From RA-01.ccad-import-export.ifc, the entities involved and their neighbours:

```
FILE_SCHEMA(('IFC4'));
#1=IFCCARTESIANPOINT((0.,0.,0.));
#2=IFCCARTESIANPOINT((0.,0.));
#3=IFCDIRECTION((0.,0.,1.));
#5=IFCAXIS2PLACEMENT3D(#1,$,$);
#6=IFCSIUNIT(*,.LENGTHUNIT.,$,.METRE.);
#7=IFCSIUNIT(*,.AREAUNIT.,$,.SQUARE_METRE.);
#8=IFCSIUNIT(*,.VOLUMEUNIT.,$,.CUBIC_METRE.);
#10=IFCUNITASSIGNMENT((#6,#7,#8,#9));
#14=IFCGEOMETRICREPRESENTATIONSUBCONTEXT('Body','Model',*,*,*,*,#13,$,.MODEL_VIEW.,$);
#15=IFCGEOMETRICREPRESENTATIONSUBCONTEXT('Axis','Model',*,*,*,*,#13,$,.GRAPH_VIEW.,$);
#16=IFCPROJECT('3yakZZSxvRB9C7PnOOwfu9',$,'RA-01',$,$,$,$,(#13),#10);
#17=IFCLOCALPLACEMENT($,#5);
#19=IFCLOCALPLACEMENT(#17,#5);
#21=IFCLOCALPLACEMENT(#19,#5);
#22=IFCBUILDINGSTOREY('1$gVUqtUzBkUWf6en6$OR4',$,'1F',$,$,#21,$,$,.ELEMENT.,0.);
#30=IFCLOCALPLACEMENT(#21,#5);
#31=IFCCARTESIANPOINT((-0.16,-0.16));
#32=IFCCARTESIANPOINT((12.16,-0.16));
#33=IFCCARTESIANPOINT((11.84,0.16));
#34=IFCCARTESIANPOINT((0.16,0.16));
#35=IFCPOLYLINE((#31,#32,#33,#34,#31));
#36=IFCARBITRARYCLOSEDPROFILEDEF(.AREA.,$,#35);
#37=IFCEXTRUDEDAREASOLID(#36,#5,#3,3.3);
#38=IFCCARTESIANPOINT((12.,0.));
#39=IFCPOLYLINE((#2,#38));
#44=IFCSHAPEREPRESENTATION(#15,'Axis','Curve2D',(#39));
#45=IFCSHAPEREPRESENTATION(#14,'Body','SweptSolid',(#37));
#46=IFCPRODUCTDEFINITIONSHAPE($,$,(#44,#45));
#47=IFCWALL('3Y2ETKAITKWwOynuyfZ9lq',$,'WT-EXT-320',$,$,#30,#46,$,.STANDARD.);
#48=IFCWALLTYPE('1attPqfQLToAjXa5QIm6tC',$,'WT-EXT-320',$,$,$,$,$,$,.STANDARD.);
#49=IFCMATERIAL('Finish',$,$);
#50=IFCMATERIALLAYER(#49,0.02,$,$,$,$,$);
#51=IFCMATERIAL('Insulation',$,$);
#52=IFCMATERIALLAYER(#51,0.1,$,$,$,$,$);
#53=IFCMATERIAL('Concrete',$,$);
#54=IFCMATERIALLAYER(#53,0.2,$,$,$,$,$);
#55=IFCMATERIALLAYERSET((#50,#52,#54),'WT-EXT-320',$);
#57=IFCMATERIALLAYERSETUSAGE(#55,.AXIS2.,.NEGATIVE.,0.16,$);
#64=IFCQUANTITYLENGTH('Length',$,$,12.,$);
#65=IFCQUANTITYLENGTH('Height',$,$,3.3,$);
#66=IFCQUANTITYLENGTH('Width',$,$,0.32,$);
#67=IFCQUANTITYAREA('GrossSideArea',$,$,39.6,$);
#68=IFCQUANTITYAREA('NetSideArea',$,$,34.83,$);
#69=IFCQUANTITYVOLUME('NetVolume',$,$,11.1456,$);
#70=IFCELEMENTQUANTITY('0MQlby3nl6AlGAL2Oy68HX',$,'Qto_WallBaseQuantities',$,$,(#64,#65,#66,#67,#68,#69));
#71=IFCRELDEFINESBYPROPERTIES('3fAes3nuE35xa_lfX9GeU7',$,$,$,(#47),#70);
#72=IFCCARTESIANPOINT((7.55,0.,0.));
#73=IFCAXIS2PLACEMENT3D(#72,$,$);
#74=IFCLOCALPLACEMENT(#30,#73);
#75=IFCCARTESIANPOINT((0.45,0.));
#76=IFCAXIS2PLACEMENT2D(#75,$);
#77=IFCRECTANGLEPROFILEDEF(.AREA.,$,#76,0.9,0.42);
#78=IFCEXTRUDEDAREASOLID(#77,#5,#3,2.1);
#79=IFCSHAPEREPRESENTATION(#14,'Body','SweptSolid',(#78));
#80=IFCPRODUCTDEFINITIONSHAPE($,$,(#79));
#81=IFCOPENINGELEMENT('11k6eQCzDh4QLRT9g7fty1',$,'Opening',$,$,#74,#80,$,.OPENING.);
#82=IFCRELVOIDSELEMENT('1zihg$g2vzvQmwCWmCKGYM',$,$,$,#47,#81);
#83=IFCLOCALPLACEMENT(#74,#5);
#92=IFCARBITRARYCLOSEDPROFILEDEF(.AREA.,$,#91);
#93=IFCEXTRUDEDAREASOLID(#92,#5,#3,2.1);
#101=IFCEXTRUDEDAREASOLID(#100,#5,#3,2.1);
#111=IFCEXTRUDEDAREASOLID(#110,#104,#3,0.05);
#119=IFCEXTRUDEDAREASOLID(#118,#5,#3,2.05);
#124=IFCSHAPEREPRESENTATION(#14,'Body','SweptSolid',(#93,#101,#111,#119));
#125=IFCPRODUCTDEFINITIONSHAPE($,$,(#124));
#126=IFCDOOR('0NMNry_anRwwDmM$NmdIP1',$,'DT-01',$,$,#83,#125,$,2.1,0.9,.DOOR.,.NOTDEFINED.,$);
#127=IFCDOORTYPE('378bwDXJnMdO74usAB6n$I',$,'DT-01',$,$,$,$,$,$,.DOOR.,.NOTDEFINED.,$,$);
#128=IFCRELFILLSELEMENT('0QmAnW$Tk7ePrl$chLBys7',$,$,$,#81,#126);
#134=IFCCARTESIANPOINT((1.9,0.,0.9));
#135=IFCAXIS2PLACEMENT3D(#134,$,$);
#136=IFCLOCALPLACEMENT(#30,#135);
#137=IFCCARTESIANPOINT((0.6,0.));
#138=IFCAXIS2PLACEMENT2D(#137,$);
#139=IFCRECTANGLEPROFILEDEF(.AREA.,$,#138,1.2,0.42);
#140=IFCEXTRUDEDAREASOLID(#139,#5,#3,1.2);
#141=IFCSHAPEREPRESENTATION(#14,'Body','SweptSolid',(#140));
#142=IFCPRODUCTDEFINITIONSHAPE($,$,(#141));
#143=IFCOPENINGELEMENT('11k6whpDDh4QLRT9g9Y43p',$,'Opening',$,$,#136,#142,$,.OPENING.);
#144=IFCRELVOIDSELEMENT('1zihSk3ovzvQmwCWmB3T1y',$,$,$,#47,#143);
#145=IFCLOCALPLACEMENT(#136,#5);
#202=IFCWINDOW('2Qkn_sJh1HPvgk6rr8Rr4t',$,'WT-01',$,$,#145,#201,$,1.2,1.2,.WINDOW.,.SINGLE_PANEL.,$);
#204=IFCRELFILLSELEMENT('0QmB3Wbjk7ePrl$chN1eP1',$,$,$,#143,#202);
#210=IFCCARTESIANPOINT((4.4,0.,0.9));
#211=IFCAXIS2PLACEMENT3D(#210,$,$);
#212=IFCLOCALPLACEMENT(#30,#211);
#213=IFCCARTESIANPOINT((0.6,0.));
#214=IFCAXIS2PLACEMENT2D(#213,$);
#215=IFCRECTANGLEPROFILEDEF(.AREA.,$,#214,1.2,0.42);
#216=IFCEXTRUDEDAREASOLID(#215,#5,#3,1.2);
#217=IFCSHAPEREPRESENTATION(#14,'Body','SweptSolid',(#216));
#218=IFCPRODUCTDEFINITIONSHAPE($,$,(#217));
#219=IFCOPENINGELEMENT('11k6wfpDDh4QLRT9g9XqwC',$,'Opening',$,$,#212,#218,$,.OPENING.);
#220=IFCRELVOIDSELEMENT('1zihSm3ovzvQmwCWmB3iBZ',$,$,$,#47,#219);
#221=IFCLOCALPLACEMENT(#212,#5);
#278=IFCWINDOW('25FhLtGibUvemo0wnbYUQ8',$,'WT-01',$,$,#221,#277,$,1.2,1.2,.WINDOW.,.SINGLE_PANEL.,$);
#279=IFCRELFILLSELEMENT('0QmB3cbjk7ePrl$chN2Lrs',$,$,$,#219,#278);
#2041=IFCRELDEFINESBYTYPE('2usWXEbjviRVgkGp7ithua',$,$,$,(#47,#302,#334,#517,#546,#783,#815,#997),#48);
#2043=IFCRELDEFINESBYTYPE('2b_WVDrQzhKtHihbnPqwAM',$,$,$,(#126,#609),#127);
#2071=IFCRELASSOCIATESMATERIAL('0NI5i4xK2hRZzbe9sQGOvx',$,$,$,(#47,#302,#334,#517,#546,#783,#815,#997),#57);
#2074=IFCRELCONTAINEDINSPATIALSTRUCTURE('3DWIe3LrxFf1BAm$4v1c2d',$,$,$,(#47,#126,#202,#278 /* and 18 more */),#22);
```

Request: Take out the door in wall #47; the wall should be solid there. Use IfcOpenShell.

```python
import ifcopenshell
import ifcopenshell.api.feature
import ifcopenshell.api.pset
import ifcopenshell.api.root
import ifcopenshell.geom
import ifcopenshell.util.element
import ifcopenshell.util.shape
import ifcopenshell.util.unit

model = ifcopenshell.open("RA-01.ccad-import-export.ifc")
area_scale = ifcopenshell.util.unit.calculate_unit_scale(model, "AREAUNIT")
volume_scale = ifcopenshell.util.unit.calculate_unit_scale(model, "VOLUMEUNIT")
settings = ifcopenshell.geom.settings()


def volume(element):
    """Net volume in cubic metres, openings subtracted."""
    shape = ifcopenshell.geom.create_shape(settings, element)
    return ifcopenshell.util.shape.get_volume(shape.geometry)


door = model.by_guid("0NMNry_anRwwDmM$NmdIP1")
opening = door.FillsVoids[0].RelatingOpeningElement
wall = opening.VoidsElements[0].RelatingBuildingElement
before = volume(wall)

ifcopenshell.api.root.remove_product(model, product=door)
ifcopenshell.api.feature.remove_feature(model, feature=opening)

after = volume(wall)
thickness = 0.32  # wall thickness in metres

# Update the wall's stored quantities.
qto = model.by_id(ifcopenshell.util.element.get_pset(wall, "Qto_WallBaseQuantities", should_inherit=False)["id"])
ifcopenshell.api.pset.edit_qto(model, qto=qto, properties={
    "NetSideArea": after / thickness / area_scale,
    "NetVolume": after / volume_scale,
})

print(f"wall volume {before:.3f} -> {after:.3f} m3")

model.write("RA-01.ccad-import-export_updated.ifc")
```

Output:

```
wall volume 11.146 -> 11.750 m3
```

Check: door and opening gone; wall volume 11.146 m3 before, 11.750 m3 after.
